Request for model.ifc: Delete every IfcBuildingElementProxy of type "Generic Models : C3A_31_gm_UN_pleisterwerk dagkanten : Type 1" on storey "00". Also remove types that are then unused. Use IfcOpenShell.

First a look at what the model holds.

```python
import ifcopenshell
import ifcopenshell.util.element

model = ifcopenshell.open("model.ifc")
print(model.schema)
storey = next(s for s in model.by_type("IfcBuildingStorey") if s.Name == "00")
proxies = [e for e in ifcopenshell.util.element.get_decomposition(storey) if e.is_a("IfcBuildingElementProxy")]
seen = {}
for e in proxies:
    element_type = ifcopenshell.util.element.get_type(e)
    name = element_type.Name if element_type not in (None, e) else None
    seen[name] = seen.get(name, 0) + 1
for name, count in sorted(seen.items(), key=str):
    print(count, "x", name)
```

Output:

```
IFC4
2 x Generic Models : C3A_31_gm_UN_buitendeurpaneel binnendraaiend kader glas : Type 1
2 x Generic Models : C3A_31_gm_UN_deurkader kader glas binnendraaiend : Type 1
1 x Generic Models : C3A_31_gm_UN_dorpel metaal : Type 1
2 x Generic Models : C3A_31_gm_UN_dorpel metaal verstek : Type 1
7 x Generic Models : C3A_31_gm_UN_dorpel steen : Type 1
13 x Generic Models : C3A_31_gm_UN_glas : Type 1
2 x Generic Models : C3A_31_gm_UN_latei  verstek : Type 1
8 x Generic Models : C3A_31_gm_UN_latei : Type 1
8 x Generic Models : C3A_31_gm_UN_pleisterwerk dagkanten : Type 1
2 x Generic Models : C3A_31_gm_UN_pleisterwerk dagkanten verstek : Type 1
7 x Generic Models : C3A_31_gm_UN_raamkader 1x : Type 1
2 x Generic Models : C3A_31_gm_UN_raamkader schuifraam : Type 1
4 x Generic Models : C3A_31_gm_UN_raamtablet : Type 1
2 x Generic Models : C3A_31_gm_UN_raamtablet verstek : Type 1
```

```python
import ifcopenshell
import ifcopenshell.api.root
import ifcopenshell.util.element

model = ifcopenshell.open("model.ifc")

storey = next(s for s in model.by_type("IfcBuildingStorey") if s.Name == "00")
proxies = [e for e in ifcopenshell.util.element.get_decomposition(storey) if e.is_a("IfcBuildingElementProxy")]
targets = [e for e in proxies if (t := ifcopenshell.util.element.get_type(e)) not in (None, e) and t.Name == "Generic Models : C3A_31_gm_UN_pleisterwerk dagkanten : Type 1"]
types = {ifcopenshell.util.element.get_type(e) for e in targets} - {None, *targets}

for e in targets:
    ifcopenshell.api.root.remove_product(model, product=e)
print(len(targets), "removed")

unused = [t for t in types if not ifcopenshell.util.element.get_types(t)]
for t in unused:
    ifcopenshell.api.root.remove_product(model, product=t)
print(len(unused), "unused types removed")

model.write("model-out.ifc")
```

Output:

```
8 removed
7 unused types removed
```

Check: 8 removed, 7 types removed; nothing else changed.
